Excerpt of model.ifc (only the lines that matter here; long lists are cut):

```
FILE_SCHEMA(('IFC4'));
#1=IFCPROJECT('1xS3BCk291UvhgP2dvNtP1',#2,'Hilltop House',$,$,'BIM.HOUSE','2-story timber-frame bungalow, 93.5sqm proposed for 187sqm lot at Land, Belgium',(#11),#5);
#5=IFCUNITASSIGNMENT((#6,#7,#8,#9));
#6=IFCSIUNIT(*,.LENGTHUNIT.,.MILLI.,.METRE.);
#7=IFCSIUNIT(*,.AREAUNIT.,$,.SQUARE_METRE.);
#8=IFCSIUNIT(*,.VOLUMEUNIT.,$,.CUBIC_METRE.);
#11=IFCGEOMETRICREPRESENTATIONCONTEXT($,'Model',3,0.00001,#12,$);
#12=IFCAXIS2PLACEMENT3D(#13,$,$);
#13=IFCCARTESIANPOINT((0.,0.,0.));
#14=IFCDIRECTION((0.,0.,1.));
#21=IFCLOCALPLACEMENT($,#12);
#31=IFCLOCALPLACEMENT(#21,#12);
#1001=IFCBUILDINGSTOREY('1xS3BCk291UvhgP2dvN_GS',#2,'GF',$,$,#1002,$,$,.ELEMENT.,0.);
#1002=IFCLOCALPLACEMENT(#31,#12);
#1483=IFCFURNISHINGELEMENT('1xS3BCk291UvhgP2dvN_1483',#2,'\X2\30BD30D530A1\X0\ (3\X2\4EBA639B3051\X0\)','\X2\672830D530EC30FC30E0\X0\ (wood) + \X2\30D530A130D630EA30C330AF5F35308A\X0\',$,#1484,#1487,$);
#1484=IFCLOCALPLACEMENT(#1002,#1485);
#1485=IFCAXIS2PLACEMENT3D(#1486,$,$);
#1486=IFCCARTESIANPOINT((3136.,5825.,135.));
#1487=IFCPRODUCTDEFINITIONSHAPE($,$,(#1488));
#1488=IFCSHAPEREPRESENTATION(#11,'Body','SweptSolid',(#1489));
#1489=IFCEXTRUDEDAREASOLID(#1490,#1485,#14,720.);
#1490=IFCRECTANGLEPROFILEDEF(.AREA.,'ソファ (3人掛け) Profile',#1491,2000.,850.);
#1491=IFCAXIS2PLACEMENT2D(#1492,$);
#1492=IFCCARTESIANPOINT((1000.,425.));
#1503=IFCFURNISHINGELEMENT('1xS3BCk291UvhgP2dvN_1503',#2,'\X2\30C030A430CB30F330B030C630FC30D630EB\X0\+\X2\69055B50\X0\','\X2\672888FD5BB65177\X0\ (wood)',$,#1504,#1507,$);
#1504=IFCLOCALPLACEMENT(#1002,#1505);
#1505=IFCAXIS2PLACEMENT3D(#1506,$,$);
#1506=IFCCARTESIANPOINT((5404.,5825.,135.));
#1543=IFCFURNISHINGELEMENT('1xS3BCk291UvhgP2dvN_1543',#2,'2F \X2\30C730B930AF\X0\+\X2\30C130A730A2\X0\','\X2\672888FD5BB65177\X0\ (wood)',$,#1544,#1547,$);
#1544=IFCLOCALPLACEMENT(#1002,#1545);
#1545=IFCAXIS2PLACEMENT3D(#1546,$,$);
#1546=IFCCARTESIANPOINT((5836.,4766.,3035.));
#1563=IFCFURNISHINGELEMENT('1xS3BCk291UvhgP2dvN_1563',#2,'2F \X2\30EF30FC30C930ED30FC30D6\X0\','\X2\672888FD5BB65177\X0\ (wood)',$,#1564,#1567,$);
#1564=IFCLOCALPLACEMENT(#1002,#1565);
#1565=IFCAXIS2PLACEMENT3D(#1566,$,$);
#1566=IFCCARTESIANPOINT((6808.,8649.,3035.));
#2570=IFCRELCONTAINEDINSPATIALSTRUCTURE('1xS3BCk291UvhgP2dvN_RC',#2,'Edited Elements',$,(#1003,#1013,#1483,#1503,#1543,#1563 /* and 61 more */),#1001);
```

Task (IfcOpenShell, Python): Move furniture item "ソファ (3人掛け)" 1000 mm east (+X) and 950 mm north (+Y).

```python
import ifcopenshell
import ifcopenshell.api.geometry
import ifcopenshell.util.placement
import ifcopenshell.util.unit

model = ifcopenshell.open("model.ifc")
unit_scale = ifcopenshell.util.unit.calculate_unit_scale(model)

item = model.by_guid("1xS3BCk291UvhgP2dvN_1483")
matrix = ifcopenshell.util.placement.get_local_placement(item.ObjectPlacement)
matrix[0, 3] += 1 / unit_scale
matrix[1, 3] += 0.95 / unit_scale
ifcopenshell.api.geometry.edit_object_placement(model, product=item, matrix=matrix, is_si=False)

print(ifcopenshell.util.placement.get_local_placement(item.ObjectPlacement).round(3) + 0.0)

model.write("model_edited.ifc")
```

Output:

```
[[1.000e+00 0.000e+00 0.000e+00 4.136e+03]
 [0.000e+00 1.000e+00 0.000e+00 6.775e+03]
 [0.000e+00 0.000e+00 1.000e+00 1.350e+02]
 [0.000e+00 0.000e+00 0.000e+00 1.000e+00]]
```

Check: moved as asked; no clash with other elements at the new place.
